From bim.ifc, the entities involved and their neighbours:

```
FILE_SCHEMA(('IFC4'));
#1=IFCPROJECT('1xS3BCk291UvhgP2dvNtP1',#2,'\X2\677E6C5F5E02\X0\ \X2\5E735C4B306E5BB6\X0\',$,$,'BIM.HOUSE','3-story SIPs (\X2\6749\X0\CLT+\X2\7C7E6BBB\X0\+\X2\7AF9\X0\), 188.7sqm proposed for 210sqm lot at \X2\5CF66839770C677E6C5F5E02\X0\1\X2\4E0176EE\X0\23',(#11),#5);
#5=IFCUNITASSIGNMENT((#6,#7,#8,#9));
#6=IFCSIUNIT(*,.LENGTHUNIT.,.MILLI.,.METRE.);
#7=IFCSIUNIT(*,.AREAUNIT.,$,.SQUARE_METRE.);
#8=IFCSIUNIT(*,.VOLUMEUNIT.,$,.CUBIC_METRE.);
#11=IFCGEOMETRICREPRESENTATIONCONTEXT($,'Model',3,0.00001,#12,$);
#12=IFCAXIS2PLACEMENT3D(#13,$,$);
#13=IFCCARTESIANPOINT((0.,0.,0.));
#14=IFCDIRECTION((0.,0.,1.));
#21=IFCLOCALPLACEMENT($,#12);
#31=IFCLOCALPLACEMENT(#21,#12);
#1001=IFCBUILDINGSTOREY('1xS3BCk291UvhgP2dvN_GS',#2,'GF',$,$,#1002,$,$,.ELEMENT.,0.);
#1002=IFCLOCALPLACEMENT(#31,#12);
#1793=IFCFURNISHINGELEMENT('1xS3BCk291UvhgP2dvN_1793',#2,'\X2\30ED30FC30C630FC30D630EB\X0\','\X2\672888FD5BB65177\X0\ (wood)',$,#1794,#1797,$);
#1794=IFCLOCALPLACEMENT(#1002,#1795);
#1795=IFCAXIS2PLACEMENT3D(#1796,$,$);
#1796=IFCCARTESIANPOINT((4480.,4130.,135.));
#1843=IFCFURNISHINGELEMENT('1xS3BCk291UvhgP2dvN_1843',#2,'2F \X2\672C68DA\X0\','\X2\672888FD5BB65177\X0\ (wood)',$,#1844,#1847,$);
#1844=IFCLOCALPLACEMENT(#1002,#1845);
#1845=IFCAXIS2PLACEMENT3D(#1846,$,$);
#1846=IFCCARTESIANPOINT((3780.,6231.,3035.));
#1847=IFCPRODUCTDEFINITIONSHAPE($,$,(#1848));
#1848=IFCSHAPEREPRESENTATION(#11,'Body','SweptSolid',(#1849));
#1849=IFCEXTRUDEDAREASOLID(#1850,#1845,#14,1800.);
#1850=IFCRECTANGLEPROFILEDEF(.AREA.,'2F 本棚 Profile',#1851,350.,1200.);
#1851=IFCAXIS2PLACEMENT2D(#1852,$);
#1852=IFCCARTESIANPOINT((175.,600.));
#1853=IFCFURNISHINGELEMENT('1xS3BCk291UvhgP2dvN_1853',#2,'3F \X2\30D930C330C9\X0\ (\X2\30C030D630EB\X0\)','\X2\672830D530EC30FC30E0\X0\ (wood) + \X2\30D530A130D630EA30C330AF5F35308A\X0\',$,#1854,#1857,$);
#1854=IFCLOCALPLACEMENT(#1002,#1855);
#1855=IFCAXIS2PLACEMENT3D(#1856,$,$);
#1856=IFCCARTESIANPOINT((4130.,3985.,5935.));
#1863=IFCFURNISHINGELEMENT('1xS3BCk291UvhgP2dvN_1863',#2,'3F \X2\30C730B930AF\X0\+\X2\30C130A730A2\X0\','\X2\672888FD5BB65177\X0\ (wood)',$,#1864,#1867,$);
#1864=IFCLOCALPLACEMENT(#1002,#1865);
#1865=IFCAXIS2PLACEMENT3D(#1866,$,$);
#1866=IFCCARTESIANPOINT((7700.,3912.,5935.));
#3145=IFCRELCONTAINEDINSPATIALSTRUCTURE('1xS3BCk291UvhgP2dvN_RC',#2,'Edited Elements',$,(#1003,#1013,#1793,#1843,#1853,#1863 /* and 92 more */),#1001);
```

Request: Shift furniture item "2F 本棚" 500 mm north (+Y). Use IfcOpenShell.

```python
import ifcopenshell
import ifcopenshell.api.geometry
import ifcopenshell.util.placement

model = ifcopenshell.open("bim.ifc")

item = model.by_guid("1xS3BCk291UvhgP2dvN_1843")
matrix = ifcopenshell.util.placement.get_local_placement(item.ObjectPlacement)
matrix[1, 3] += 500.0
ifcopenshell.api.geometry.edit_object_placement(model, product=item, matrix=matrix, is_si=False)

print(ifcopenshell.util.placement.get_local_placement(item.ObjectPlacement).round(3) + 0.0)

model.write("bim_rev.ifc")
```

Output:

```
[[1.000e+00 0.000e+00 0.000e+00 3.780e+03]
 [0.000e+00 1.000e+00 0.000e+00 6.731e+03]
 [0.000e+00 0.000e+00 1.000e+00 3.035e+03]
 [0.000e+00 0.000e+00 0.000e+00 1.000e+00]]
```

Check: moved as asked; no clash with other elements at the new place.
